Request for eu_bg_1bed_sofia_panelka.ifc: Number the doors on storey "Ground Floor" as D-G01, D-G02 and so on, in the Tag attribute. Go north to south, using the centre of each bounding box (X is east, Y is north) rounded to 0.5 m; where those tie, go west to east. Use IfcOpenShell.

First a look at what the model holds.

```python
import ifcopenshell
import ifcopenshell.util.element
import ifcopenshell.util.placement

model = ifcopenshell.open("eu_bg_1bed_sofia_panelka.ifc")
print(model.schema)
storey = next(s for s in model.by_type("IfcBuildingStorey") if s.Name == "Ground Floor")
doors = [e for e in ifcopenshell.util.element.get_decomposition(storey) if e.is_a("IfcDoor")]
for e in sorted(doors, key=lambda e: e.id()):
    origin = ifcopenshell.util.placement.get_local_placement(e.ObjectPlacement)[:3, 3]
    print(e.id(), e.Tag, e.Name, origin.round(2) + 0.0, sep=" | ")
```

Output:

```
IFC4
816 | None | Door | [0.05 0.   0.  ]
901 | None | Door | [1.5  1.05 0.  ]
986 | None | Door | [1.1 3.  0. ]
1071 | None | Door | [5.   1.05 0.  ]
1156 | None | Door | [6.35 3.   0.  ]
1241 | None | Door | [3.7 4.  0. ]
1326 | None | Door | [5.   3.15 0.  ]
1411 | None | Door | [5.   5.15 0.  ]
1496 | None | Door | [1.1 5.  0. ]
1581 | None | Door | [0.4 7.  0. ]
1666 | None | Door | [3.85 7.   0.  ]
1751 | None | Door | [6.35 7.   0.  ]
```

```python
import ifcopenshell
import ifcopenshell.geom
import ifcopenshell.util.element
import ifcopenshell.util.shape

model = ifcopenshell.open("eu_bg_1bed_sofia_panelka.ifc")
settings = ifcopenshell.geom.settings()
settings.set("use-world-coords", True)


def centre(element):
    shape = ifcopenshell.geom.create_shape(settings, element)
    return ifcopenshell.util.shape.get_bbox_centroid(shape.geometry)


storey = next(s for s in model.by_type("IfcBuildingStorey") if s.Name == "Ground Floor")
doors = [e for e in ifcopenshell.util.element.get_decomposition(storey) if e.is_a("IfcDoor")]

# Insertion points can sit at a corner or the storey origin, so sort by the geometry (in metres).
centres = {e: centre(e) for e in doors}
doors.sort(key=lambda e: (-round(centres[e][1] / 0.5), centres[e][0]))

for i, e in enumerate(doors, start=1):
    number = f"D-G{i:02d}"
    e.Tag = number
    print(e.id(), number)

model.write("eu_bg_1bed_sofia_panelka_rev.ifc")
```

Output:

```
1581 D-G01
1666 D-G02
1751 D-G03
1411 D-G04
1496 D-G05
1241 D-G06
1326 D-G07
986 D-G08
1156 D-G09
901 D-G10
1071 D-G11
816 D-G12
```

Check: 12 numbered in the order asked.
